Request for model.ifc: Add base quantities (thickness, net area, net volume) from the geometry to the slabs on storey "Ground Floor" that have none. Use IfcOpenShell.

First a look at what the model holds.

```python
import ifcopenshell
import ifcopenshell.util.element
import ifcopenshell.util.unit

model = ifcopenshell.open("model.ifc")
print(model.schema)
for unit_type in ("LENGTHUNIT", "AREAUNIT", "VOLUMEUNIT"):
    print(unit_type, ifcopenshell.util.unit.calculate_unit_scale(model, unit_type))
storey = next(s for s in model.by_type("IfcBuildingStorey") if s.Name == "Ground Floor")
slabs = [e for e in ifcopenshell.util.element.get_decomposition(storey) if e.is_a("IfcSlab")]
for e in sorted(slabs, key=lambda e: e.id()):
    print(e.id(), e.is_a(), e.Name, list(ifcopenshell.util.element.get_psets(e, qtos_only=True)), sep=" | ")
```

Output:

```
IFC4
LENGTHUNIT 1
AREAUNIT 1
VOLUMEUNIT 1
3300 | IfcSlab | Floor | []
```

```python
import ifcopenshell
import ifcopenshell.api.pset
import ifcopenshell.geom
import ifcopenshell.util.element
import ifcopenshell.util.shape
import ifcopenshell.util.unit

model = ifcopenshell.open("model.ifc")
unit_scale = ifcopenshell.util.unit.calculate_unit_scale(model)
area_scale = ifcopenshell.util.unit.calculate_unit_scale(model, "AREAUNIT")
volume_scale = ifcopenshell.util.unit.calculate_unit_scale(model, "VOLUMEUNIT")
settings = ifcopenshell.geom.settings()

storey = next(s for s in model.by_type("IfcBuildingStorey") if s.Name == "Ground Floor")
slabs = [e for e in ifcopenshell.util.element.get_decomposition(storey) if e.is_a("IfcSlab")]

for e in sorted(slabs, key=lambda e: e.id()):
    if ifcopenshell.util.element.get_psets(e, qtos_only=True, should_inherit=False):
        continue
    # Geometry comes back in metres, in the element's own axes.
    shape = ifcopenshell.geom.create_shape(settings, e)
    values = {
        "Width": ifcopenshell.util.shape.get_z(shape.geometry) / unit_scale,
        "NetArea": ifcopenshell.util.shape.get_footprint_area(shape.geometry) / area_scale,
        "NetVolume": ifcopenshell.util.shape.get_volume(shape.geometry) / volume_scale,
    }
    qto = ifcopenshell.api.pset.add_qto(model, product=e, name="Qto_SlabBaseQuantities")
    ifcopenshell.api.pset.edit_qto(model, qto=qto, properties=values)
    print(e.id(), {k: round(v, 3) for k, v in values.items()})

model.write("model_updated.ifc")
```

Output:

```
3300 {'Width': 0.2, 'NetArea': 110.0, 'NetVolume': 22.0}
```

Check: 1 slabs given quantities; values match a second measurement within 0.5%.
